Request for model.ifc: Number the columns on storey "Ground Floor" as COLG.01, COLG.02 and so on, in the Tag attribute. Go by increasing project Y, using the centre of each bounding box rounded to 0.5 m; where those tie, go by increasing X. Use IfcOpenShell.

First a look at what the model holds.

```python
import ifcopenshell
import ifcopenshell.util.element
import ifcopenshell.util.placement

model = ifcopenshell.open("model.ifc")
print(model.schema)
storey = next(s for s in model.by_type("IfcBuildingStorey") if s.Name == "Ground Floor")
columns = [e for e in ifcopenshell.util.element.get_decomposition(storey) if e.is_a("IfcColumn")]
for e in sorted(columns, key=lambda e: e.id()):
    origin = ifcopenshell.util.placement.get_local_placement(e.ObjectPlacement)[:3, 3]
    print(e.id(), e.Tag, e.Name, origin.round(2) + 0.0, sep=" | ")
```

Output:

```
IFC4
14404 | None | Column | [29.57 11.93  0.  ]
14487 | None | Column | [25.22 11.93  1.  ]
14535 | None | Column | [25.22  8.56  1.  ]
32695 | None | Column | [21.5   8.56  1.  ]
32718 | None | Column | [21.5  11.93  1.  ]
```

```python
import ifcopenshell
import ifcopenshell.geom
import ifcopenshell.util.element
import ifcopenshell.util.shape

model = ifcopenshell.open("model.ifc")
settings = ifcopenshell.geom.settings()
settings.set("use-world-coords", True)


def centre(element):
    shape = ifcopenshell.geom.create_shape(settings, element)
    return ifcopenshell.util.shape.get_bbox_centroid(shape.geometry)


storey = next(s for s in model.by_type("IfcBuildingStorey") if s.Name == "Ground Floor")
columns = [e for e in ifcopenshell.util.element.get_decomposition(storey) if e.is_a("IfcColumn")]

# Insertion points can sit at a corner or the storey origin, so sort by the geometry (in metres).
centres = {e: centre(e) for e in columns}
columns.sort(key=lambda e: (round(centres[e][1] / 0.5), centres[e][0]))

for i, e in enumerate(columns, start=1):
    number = f"COLG.{i:02d}"
    e.Tag = number
    print(e.id(), number)

model.write("model-out.ifc")
```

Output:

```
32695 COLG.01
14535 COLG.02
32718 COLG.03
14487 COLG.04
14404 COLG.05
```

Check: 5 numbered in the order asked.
